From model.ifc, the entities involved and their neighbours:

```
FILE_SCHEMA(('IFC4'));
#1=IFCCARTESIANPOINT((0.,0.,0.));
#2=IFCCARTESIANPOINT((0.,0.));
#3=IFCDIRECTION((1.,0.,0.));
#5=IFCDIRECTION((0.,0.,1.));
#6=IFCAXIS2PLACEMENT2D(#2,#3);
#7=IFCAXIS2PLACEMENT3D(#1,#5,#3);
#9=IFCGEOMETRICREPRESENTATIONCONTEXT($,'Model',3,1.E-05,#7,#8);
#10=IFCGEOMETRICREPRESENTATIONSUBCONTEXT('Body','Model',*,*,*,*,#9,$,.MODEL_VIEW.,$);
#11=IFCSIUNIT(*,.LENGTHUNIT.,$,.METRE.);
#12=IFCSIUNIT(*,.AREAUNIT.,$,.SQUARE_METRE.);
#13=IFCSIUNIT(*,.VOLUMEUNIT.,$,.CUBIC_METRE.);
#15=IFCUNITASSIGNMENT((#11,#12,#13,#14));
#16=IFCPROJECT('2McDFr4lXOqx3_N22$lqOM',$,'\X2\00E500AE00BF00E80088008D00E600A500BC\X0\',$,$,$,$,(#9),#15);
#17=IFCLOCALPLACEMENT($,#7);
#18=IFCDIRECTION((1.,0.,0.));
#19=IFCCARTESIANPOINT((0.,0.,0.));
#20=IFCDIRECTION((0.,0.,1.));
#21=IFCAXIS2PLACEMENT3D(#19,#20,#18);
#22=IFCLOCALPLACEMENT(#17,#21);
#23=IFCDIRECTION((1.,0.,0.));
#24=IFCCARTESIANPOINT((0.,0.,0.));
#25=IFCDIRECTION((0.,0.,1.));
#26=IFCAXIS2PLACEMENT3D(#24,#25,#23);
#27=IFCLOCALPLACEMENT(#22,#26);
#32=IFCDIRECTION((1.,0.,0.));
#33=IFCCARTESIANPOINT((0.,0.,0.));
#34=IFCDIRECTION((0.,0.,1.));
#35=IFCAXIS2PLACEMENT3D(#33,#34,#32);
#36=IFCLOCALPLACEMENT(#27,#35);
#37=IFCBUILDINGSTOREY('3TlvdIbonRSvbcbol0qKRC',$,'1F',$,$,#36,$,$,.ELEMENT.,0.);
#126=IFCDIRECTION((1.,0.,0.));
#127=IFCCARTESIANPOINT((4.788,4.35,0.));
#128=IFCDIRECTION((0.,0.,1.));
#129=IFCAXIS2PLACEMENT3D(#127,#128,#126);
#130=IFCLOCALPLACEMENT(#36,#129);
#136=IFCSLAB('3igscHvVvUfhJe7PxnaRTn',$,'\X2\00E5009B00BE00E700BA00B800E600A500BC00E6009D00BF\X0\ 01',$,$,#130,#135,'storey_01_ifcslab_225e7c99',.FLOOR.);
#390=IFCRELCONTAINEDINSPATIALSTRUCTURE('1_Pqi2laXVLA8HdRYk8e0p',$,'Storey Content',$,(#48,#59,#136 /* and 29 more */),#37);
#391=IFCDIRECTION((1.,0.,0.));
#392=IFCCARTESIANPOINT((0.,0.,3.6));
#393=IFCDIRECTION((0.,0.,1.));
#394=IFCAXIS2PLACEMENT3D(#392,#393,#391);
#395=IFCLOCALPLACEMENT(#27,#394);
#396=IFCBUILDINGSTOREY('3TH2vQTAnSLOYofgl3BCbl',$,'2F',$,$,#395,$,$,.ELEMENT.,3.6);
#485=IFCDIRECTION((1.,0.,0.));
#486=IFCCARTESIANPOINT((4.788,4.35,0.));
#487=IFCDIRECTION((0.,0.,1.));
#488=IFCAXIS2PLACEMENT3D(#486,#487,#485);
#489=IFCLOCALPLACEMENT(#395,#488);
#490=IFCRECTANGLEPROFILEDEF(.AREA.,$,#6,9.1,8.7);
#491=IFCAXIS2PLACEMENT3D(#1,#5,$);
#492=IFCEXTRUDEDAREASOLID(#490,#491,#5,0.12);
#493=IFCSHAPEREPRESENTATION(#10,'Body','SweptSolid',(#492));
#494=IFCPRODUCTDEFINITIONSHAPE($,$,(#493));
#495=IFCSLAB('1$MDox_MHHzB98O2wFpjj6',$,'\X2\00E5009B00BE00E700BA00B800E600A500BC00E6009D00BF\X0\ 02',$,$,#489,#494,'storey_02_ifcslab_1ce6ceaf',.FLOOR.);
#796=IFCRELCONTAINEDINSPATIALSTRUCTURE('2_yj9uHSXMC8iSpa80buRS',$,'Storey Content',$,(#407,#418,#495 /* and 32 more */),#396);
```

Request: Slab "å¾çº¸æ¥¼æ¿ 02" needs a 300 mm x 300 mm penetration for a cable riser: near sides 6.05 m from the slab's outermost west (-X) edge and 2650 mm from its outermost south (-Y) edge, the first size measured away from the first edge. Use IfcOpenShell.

```python
import numpy as np
import ifcopenshell
import ifcopenshell.api.feature
import ifcopenshell.api.geometry
import ifcopenshell.api.root
import ifcopenshell.geom
import ifcopenshell.util.placement
import ifcopenshell.util.representation
import ifcopenshell.util.shape
import ifcopenshell.util.unit

model = ifcopenshell.open("model.ifc")
unit_scale = ifcopenshell.util.unit.calculate_unit_scale(model)
settings = ifcopenshell.geom.settings()


def volume(element):
    """Net volume in cubic metres, openings subtracted."""
    shape = ifcopenshell.geom.create_shape(settings, element)
    return ifcopenshell.util.shape.get_volume(shape.geometry)


slab = model.by_guid("1$MDox_MHHzB98O2wFpjj6")
before = volume(slab)

# Extent in the slab's own axes, in metres. The edges named are its -X and -Y sides.
slab_shape = ifcopenshell.geom.create_shape(settings, slab)
vertices = ifcopenshell.util.shape.get_vertices(slab_shape.geometry)
x_min, y_min, bottom = vertices.min(axis=0)
top = vertices[:, 2].max()

opening = ifcopenshell.api.root.create_entity(model, ifc_class="IfcOpeningElement", name="Cable riser opening", predefined_type="OPENING")
context = ifcopenshell.util.representation.get_context(model, "Model", "Body", "MODEL_VIEW")
width, depth = 0.3, 0.3
outline = [(0.0, 0.0), (width, 0.0), (width, depth), (0.0, depth), (0.0, 0.0)]
# Overshoot both faces by 50 mm so the cut is clean.
shape = ifcopenshell.api.geometry.add_slab_representation(
    model, context=context, depth=top - bottom + 0.1, polyline=outline
)
ifcopenshell.api.geometry.assign_representation(model, product=opening, representation=shape)

matrix = ifcopenshell.util.placement.get_local_placement(slab.ObjectPlacement)
matrix[:, 3] = matrix @ np.append(np.array([x_min + 6.05, y_min + 2.65, bottom - 0.05]) / unit_scale, 1.0)
ifcopenshell.api.geometry.edit_object_placement(model, product=opening, matrix=matrix, is_si=False)
ifcopenshell.api.feature.add_feature(model, feature=opening, element=slab)

after = volume(slab)

print(f"slab volume {before:.3f} -> {after:.3f} m3")

model.write("model-out.ifc")
```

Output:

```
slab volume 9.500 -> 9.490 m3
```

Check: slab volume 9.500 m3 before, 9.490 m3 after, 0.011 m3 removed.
